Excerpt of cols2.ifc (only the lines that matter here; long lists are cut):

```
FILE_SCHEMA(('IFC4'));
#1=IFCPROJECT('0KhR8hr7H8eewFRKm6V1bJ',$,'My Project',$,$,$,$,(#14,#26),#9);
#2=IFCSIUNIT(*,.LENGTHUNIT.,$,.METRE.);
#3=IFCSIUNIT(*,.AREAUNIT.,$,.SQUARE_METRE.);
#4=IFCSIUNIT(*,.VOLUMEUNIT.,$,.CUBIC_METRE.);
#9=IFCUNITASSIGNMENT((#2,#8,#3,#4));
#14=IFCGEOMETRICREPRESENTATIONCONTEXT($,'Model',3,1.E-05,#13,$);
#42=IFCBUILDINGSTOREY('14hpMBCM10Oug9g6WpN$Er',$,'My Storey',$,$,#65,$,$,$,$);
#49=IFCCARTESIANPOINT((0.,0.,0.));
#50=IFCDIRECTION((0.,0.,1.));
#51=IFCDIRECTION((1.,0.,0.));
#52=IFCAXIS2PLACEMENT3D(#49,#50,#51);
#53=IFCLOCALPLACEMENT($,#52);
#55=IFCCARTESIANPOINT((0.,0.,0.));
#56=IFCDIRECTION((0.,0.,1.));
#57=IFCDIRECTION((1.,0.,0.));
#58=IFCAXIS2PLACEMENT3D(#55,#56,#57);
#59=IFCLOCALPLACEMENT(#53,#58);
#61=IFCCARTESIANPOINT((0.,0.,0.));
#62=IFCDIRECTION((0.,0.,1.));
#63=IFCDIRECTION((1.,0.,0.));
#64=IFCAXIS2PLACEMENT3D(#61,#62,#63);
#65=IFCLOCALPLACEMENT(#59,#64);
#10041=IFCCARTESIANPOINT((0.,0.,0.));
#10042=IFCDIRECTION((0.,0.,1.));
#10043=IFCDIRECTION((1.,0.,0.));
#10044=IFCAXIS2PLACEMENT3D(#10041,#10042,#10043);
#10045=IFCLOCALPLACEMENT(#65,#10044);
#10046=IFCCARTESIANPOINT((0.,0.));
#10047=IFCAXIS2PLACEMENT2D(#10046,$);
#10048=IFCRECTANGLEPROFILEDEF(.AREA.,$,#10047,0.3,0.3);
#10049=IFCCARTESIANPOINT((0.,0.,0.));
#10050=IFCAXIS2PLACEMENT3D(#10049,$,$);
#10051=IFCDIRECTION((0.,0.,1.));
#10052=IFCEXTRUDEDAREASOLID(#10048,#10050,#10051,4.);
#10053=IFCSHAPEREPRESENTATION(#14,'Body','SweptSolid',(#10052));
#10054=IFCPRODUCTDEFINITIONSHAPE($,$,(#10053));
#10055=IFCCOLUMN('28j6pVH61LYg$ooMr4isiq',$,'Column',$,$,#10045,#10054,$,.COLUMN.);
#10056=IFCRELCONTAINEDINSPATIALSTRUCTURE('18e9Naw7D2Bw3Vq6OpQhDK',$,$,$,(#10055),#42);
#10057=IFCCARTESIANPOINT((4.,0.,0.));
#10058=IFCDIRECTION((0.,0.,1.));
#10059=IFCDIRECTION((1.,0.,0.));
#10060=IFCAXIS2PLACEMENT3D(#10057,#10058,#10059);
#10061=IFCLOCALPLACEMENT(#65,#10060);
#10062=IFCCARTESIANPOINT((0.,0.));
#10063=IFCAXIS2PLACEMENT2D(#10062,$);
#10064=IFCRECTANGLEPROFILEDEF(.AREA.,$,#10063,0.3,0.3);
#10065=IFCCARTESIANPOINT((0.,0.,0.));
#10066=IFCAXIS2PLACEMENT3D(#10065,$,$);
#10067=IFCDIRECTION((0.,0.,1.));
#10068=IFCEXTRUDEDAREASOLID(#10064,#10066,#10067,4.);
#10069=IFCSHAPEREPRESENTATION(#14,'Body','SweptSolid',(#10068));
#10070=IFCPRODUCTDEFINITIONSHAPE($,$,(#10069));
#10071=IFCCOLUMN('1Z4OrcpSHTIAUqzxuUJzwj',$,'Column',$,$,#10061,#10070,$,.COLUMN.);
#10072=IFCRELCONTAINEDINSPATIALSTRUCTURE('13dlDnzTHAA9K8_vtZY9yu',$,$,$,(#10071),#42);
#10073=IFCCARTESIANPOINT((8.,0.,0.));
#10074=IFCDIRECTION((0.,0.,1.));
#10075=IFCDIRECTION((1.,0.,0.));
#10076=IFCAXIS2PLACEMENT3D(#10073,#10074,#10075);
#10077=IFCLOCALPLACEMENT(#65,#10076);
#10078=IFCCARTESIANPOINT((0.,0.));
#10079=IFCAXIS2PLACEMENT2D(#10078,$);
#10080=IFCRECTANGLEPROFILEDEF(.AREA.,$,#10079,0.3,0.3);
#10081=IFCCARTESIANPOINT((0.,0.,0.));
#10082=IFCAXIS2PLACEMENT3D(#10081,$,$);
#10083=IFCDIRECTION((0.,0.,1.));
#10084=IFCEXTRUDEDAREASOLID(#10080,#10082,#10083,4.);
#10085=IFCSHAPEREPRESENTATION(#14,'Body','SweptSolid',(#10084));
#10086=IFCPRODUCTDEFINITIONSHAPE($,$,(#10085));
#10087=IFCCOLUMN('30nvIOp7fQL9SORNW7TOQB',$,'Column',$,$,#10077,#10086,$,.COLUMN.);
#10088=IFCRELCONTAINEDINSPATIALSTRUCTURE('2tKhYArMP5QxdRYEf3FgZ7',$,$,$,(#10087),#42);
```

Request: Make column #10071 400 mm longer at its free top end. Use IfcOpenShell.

```python
import ifcopenshell
import ifcopenshell.util.unit

model = ifcopenshell.open("cols2.ifc")
unit_scale = ifcopenshell.util.unit.calculate_unit_scale(model)

member = model.by_guid("1Z4OrcpSHTIAUqzxuUJzwj")
change = 0.4 / unit_scale

# The extrusion runs towards the end named, so only its depth changes.
body = next(r for r in member.Representation.Representations if r.RepresentationIdentifier == "Body")
solid = body.Items[0]
old_length = solid.Depth
solid.Depth += change

print(f"length {old_length:g} -> {solid.Depth:g}")

model.write("cols2_v2.ifc")
```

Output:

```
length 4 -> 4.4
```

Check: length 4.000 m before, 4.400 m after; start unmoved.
